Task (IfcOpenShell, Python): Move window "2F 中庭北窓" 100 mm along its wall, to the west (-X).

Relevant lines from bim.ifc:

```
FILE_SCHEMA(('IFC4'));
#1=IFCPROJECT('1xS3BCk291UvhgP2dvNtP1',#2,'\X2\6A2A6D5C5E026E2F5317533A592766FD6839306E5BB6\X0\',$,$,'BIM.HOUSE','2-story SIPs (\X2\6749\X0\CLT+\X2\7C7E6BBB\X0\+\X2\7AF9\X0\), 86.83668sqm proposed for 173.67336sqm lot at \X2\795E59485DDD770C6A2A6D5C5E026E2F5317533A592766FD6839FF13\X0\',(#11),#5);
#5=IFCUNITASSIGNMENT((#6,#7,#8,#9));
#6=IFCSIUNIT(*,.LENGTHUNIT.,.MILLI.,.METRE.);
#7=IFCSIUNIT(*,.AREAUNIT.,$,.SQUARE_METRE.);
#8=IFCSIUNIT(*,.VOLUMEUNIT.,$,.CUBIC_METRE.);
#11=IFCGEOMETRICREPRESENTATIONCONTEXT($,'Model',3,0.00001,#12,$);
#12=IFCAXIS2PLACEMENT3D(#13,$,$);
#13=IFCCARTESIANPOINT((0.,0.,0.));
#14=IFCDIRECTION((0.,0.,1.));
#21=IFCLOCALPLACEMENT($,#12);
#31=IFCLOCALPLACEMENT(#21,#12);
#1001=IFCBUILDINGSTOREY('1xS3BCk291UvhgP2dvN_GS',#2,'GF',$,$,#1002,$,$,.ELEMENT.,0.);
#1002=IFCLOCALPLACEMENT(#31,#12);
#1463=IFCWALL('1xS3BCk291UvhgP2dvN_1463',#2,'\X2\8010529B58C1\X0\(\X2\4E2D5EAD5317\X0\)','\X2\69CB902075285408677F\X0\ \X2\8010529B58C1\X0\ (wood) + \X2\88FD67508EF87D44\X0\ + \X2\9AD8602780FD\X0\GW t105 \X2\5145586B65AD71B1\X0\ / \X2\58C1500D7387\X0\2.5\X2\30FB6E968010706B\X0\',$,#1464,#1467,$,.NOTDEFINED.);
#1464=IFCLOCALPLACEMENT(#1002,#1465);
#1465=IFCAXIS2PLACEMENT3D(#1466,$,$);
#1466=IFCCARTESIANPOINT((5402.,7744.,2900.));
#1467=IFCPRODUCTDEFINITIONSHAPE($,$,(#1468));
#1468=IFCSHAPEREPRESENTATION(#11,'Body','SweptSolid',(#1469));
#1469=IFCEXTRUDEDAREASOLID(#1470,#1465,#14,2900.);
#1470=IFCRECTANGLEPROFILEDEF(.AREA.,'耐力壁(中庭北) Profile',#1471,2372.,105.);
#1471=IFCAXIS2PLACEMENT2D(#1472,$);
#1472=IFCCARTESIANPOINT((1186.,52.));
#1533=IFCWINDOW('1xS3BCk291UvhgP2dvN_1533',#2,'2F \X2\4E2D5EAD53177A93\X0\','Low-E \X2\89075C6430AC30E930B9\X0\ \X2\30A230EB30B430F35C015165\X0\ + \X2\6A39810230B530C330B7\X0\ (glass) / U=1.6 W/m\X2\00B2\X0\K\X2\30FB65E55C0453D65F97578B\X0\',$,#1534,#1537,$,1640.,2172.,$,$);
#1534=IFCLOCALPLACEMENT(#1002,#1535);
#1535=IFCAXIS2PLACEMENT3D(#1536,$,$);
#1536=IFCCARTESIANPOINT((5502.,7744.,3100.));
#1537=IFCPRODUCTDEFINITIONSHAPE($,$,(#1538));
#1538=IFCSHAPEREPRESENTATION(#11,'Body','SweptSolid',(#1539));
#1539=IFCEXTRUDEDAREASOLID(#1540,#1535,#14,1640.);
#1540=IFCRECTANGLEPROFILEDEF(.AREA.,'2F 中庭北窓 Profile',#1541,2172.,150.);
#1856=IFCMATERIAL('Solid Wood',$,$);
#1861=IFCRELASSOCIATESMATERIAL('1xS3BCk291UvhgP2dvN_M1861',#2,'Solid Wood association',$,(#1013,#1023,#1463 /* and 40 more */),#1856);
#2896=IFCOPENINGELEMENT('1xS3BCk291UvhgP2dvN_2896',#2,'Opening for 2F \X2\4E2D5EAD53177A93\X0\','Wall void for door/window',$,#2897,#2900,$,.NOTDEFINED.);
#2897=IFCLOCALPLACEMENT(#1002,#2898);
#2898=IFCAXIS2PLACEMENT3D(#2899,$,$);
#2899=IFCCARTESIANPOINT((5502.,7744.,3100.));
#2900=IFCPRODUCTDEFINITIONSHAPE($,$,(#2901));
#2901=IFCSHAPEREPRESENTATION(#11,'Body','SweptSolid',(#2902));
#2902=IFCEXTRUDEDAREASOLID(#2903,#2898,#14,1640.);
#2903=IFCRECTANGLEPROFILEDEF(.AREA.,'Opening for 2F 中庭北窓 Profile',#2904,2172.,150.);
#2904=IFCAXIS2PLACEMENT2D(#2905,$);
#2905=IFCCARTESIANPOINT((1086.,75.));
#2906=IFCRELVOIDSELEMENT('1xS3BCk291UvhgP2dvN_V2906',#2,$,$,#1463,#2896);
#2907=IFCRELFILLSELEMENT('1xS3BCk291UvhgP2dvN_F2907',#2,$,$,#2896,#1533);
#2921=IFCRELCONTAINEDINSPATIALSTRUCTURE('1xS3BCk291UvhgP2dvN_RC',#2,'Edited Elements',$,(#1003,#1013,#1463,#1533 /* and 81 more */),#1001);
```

```python
import ifcopenshell
import ifcopenshell.api.geometry
import ifcopenshell.util.placement

model = ifcopenshell.open("bim.ifc")

window = model.by_id(1533)
opening = window.FillsVoids[0].RelatingOpeningElement
wall = opening.VoidsElements[0].RelatingBuildingElement

wall_matrix = ifcopenshell.util.placement.get_local_placement(wall.ObjectPlacement)
shift = wall_matrix[:3, 0] * -100.0
before = ifcopenshell.util.placement.get_local_placement(window.ObjectPlacement)[:3, 3].copy()

# The window is not placed relative to its opening, so move both.
for product in (opening, window):
    matrix = ifcopenshell.util.placement.get_local_placement(product.ObjectPlacement)
    matrix[:3, 3] += shift
    ifcopenshell.api.geometry.edit_object_placement(model, product=product, matrix=matrix, is_si=False)

after = ifcopenshell.util.placement.get_local_placement(window.ObjectPlacement)[:3, 3]
print("window moved by", (after - before).round(3) + 0.0)

model.write("bim_edited.ifc")
```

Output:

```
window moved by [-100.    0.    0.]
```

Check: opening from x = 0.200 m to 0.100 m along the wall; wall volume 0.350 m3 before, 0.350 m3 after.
